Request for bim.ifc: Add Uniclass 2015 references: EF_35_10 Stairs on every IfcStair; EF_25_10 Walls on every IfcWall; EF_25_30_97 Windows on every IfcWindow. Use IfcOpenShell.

First a look at what the model holds.

```python
import ifcopenshell

model = ifcopenshell.open("bim.ifc")
print(model.schema)
print("classifications:", [c.Name for c in model.by_type("IfcClassification")])
for ifc_class in ("IfcDoor", "IfcRoof", "IfcStair", "IfcWall", "IfcWindow"):
    print(ifc_class, len(model.by_type(ifc_class)))
```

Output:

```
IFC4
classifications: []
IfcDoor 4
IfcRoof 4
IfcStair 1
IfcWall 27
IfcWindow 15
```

```python
import ifcopenshell
import ifcopenshell.api.classification

model = ifcopenshell.open("bim.ifc")

system = ifcopenshell.api.classification.add_classification(model, classification="Uniclass 2015")

codes = {
    "IfcStair": ("EF_35_10", "Stairs"),
    "IfcWall": ("EF_25_10", "Walls"),
    "IfcWindow": ("EF_25_30_97", "Windows"),
}
for ifc_class, (code, name) in codes.items():
    products = model.by_type(ifc_class)
    ifcopenshell.api.classification.add_reference(
        model, products=products, classification=system, identification=code, name=name
    )
    print(code, len(products))

model.write("bim-out.ifc")
```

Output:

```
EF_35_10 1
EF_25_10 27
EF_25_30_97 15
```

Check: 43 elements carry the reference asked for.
